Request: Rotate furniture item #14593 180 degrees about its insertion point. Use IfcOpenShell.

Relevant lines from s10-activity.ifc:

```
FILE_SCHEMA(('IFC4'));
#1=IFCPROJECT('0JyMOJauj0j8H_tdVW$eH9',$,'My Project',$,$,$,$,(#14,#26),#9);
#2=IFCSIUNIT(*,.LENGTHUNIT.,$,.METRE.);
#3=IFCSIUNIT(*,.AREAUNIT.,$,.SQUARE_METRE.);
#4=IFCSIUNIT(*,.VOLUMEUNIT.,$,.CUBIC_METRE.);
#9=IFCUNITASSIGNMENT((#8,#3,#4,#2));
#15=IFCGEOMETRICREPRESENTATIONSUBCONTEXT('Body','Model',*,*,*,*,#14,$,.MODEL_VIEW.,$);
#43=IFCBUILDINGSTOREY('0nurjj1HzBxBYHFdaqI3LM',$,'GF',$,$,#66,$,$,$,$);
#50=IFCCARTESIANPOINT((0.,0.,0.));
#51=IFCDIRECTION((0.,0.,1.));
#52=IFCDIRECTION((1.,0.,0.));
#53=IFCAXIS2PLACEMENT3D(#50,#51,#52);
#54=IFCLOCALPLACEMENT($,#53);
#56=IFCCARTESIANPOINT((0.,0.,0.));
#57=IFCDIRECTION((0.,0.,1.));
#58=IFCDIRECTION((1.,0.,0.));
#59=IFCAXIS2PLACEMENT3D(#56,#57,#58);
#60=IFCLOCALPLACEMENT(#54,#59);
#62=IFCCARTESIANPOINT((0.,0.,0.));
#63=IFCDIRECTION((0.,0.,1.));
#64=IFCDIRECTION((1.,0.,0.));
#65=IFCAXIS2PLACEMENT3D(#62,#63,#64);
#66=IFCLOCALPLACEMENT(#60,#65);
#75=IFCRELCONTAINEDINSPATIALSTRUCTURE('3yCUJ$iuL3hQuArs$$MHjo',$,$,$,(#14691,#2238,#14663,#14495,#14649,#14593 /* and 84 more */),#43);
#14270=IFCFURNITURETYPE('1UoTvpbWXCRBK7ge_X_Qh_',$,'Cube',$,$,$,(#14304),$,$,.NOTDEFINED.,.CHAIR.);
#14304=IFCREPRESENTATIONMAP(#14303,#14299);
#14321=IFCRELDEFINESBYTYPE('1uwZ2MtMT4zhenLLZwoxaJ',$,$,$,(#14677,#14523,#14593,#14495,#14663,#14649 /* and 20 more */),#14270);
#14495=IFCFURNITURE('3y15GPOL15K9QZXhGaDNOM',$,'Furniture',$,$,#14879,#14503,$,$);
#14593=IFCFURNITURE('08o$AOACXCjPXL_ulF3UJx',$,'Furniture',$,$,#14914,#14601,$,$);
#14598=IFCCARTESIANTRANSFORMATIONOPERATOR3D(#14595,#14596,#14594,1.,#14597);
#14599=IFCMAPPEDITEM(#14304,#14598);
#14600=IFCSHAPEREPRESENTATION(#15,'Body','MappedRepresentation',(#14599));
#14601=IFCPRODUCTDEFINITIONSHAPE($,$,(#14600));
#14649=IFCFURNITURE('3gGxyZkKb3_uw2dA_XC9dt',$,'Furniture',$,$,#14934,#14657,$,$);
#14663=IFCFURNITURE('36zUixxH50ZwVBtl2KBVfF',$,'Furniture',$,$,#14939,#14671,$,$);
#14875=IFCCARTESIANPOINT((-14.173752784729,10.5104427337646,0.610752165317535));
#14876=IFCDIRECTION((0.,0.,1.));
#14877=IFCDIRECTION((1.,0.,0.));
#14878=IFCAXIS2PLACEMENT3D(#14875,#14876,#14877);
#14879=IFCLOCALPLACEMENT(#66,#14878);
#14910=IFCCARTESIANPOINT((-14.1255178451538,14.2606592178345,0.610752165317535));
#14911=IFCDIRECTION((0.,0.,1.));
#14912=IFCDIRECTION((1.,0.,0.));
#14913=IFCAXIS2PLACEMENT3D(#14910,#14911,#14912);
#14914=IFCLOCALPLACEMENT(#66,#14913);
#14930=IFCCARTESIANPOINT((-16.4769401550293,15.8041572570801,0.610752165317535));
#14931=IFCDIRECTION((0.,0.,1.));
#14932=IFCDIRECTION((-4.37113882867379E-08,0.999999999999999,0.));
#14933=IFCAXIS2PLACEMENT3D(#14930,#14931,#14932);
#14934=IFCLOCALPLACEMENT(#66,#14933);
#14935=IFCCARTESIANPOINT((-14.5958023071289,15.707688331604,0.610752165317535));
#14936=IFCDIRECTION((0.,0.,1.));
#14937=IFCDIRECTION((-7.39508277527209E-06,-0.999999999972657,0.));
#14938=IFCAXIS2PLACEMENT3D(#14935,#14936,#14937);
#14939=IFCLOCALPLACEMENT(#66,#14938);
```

```python
import ifcopenshell
import ifcopenshell.api.geometry
import ifcopenshell.util.placement

model = ifcopenshell.open("s10-activity.ifc")

item = model.by_id(14593)
matrix = ifcopenshell.util.placement.get_local_placement(item.ObjectPlacement)
matrix = matrix @ ifcopenshell.util.placement.rotation(180, "Z")
ifcopenshell.api.geometry.edit_object_placement(model, product=item, matrix=matrix, is_si=False)

print(ifcopenshell.util.placement.get_local_placement(item.ObjectPlacement).round(3) + 0.0)

model.write("s10-activity_v2.ifc")
```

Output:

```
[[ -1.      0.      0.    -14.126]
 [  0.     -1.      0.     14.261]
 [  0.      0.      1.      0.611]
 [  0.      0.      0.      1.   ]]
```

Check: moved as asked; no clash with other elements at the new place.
